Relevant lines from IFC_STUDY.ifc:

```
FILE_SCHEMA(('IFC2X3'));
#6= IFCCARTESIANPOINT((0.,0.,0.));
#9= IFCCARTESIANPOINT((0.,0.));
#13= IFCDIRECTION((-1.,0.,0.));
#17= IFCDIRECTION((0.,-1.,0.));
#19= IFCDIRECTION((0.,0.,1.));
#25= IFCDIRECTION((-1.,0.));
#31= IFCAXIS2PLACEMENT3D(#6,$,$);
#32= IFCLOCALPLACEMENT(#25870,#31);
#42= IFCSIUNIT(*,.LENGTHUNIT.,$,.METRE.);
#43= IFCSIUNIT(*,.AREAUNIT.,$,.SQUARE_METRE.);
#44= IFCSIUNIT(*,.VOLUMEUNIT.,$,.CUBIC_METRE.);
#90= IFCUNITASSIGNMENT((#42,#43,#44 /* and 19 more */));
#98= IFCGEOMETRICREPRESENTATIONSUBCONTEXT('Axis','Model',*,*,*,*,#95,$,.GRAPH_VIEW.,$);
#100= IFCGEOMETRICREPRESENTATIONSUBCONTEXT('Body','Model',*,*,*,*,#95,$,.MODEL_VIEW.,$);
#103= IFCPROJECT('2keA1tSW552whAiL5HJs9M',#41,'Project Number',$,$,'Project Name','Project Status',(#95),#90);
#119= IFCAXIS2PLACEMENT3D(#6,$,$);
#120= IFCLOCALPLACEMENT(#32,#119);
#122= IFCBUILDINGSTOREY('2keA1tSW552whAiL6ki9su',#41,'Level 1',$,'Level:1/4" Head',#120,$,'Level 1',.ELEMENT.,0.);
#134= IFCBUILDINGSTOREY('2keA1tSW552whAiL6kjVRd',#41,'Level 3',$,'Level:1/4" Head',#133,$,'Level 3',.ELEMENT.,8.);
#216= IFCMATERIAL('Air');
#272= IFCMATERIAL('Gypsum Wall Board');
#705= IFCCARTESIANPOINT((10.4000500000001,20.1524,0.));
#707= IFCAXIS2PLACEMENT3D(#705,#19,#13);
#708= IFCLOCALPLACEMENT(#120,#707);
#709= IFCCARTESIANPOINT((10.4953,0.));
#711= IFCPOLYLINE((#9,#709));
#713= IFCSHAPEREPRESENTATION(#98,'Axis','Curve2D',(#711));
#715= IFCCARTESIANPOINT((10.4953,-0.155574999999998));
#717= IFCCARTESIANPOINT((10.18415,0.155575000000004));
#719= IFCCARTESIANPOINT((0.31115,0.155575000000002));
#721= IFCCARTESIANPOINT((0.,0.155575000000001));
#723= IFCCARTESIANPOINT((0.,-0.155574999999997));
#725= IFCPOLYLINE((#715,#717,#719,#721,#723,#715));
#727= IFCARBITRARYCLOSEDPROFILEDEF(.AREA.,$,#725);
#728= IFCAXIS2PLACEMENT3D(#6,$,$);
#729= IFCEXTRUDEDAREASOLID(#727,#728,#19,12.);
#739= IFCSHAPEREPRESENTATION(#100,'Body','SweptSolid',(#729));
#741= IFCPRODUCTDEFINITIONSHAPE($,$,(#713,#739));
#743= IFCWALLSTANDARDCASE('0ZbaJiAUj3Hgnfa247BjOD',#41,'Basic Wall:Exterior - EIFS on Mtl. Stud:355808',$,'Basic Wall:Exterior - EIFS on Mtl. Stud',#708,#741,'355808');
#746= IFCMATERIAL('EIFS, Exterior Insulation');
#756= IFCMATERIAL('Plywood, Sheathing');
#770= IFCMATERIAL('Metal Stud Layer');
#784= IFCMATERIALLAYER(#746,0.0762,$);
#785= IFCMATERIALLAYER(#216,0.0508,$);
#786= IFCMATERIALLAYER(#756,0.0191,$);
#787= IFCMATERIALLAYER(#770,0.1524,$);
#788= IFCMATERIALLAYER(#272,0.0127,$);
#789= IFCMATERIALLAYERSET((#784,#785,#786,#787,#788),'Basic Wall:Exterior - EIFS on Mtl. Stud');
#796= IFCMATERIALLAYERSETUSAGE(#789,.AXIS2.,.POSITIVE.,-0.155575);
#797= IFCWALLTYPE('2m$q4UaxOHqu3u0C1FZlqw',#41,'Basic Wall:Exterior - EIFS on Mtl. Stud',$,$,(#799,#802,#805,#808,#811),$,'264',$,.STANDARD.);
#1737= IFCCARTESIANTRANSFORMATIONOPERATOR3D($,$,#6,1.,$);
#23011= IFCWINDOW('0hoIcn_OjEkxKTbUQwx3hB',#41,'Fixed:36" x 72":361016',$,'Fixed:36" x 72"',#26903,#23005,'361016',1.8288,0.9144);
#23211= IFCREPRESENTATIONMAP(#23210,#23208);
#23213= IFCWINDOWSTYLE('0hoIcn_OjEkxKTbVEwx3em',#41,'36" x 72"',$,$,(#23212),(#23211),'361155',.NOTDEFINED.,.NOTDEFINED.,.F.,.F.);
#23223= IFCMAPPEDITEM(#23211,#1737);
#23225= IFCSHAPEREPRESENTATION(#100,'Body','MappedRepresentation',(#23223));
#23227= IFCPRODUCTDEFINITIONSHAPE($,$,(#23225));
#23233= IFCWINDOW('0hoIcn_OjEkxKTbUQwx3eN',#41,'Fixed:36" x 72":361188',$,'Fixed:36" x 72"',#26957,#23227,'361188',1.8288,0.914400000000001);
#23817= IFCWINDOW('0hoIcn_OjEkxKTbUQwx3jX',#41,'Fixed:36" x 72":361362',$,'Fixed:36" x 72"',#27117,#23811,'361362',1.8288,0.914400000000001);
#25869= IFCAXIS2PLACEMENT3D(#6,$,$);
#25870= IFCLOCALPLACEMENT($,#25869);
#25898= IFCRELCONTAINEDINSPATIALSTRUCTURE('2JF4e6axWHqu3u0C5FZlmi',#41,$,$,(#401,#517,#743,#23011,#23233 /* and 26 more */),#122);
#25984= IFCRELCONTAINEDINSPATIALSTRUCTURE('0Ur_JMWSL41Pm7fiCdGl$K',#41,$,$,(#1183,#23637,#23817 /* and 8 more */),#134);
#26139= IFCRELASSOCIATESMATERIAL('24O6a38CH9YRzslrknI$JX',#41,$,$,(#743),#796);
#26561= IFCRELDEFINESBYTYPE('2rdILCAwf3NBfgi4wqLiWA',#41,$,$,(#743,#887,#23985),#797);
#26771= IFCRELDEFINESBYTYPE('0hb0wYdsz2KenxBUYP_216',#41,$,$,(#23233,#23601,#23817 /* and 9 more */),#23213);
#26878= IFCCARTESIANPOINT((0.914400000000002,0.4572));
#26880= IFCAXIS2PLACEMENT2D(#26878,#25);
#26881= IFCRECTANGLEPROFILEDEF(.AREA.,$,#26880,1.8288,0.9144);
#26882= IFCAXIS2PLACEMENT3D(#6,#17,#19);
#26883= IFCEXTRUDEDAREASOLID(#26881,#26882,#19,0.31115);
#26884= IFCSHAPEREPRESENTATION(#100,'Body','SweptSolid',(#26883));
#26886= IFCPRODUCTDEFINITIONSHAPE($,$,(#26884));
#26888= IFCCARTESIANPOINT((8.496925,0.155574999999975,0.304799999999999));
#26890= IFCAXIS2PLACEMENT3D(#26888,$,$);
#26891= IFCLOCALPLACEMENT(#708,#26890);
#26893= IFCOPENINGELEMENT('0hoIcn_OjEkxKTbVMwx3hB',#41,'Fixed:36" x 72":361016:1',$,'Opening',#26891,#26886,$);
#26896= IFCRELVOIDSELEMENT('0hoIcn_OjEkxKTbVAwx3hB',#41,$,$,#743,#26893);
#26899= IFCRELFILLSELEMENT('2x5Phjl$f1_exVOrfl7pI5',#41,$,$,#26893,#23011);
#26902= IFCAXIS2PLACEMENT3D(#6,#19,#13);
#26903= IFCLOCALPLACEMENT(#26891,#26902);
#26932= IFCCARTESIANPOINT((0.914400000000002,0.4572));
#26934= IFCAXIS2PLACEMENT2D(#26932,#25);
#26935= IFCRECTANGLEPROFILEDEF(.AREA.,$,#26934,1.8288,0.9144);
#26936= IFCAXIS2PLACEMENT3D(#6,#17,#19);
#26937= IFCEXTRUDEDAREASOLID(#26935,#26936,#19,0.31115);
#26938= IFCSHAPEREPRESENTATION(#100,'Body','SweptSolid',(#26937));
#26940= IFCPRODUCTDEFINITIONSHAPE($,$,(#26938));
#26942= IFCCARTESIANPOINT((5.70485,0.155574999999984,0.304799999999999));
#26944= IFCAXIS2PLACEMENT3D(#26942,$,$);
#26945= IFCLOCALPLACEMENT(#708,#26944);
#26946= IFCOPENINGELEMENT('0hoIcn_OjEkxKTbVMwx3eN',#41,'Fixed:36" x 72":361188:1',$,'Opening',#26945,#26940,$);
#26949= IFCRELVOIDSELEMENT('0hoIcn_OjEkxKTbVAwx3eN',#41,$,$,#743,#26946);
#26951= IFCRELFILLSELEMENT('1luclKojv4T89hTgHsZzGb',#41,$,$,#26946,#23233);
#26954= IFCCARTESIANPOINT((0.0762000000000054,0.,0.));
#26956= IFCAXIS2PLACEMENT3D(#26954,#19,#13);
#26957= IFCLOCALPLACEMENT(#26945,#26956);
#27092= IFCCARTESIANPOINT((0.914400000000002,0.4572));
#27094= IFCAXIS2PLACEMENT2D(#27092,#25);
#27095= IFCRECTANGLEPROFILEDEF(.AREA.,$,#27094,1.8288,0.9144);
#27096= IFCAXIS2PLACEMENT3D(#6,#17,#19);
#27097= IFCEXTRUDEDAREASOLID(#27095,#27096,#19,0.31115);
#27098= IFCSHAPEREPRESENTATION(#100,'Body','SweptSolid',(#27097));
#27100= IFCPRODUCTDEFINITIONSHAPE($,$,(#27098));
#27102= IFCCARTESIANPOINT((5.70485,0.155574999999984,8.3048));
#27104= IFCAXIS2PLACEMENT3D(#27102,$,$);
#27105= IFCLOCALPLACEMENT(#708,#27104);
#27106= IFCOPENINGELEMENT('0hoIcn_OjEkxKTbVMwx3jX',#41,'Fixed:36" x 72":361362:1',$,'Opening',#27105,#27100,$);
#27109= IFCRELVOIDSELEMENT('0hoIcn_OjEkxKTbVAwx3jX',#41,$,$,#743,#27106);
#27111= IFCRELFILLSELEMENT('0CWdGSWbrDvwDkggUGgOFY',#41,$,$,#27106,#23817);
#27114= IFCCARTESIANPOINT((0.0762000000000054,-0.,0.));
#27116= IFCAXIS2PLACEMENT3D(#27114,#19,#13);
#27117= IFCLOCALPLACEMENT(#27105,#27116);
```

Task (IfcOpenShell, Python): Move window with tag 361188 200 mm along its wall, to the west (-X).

```python
import ifcopenshell
import ifcopenshell.api.geometry
import ifcopenshell.util.placement
import ifcopenshell.util.unit

model = ifcopenshell.open("IFC_STUDY.ifc")
unit_scale = ifcopenshell.util.unit.calculate_unit_scale(model)

window = model.by_id(23233)
opening = window.FillsVoids[0].RelatingOpeningElement
wall = opening.VoidsElements[0].RelatingBuildingElement

wall_matrix = ifcopenshell.util.placement.get_local_placement(wall.ObjectPlacement)
shift = wall_matrix[:3, 0] * 0.2 / unit_scale
before = ifcopenshell.util.placement.get_local_placement(window.ObjectPlacement)[:3, 3].copy()

# The window is placed relative to its opening, so it follows when the opening moves.
matrix = ifcopenshell.util.placement.get_local_placement(opening.ObjectPlacement)
matrix[:3, 3] += shift
ifcopenshell.api.geometry.edit_object_placement(
    model, product=opening, matrix=matrix, is_si=False, should_transform_children=True
)

after = ifcopenshell.util.placement.get_local_placement(window.ObjectPlacement)[:3, 3]
print("window moved by", (after - before).round(3) + 0.0)

model.write("IFC_STUDY-out.ifc")
```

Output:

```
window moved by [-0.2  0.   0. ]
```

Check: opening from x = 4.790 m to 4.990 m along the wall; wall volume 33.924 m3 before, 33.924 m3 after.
